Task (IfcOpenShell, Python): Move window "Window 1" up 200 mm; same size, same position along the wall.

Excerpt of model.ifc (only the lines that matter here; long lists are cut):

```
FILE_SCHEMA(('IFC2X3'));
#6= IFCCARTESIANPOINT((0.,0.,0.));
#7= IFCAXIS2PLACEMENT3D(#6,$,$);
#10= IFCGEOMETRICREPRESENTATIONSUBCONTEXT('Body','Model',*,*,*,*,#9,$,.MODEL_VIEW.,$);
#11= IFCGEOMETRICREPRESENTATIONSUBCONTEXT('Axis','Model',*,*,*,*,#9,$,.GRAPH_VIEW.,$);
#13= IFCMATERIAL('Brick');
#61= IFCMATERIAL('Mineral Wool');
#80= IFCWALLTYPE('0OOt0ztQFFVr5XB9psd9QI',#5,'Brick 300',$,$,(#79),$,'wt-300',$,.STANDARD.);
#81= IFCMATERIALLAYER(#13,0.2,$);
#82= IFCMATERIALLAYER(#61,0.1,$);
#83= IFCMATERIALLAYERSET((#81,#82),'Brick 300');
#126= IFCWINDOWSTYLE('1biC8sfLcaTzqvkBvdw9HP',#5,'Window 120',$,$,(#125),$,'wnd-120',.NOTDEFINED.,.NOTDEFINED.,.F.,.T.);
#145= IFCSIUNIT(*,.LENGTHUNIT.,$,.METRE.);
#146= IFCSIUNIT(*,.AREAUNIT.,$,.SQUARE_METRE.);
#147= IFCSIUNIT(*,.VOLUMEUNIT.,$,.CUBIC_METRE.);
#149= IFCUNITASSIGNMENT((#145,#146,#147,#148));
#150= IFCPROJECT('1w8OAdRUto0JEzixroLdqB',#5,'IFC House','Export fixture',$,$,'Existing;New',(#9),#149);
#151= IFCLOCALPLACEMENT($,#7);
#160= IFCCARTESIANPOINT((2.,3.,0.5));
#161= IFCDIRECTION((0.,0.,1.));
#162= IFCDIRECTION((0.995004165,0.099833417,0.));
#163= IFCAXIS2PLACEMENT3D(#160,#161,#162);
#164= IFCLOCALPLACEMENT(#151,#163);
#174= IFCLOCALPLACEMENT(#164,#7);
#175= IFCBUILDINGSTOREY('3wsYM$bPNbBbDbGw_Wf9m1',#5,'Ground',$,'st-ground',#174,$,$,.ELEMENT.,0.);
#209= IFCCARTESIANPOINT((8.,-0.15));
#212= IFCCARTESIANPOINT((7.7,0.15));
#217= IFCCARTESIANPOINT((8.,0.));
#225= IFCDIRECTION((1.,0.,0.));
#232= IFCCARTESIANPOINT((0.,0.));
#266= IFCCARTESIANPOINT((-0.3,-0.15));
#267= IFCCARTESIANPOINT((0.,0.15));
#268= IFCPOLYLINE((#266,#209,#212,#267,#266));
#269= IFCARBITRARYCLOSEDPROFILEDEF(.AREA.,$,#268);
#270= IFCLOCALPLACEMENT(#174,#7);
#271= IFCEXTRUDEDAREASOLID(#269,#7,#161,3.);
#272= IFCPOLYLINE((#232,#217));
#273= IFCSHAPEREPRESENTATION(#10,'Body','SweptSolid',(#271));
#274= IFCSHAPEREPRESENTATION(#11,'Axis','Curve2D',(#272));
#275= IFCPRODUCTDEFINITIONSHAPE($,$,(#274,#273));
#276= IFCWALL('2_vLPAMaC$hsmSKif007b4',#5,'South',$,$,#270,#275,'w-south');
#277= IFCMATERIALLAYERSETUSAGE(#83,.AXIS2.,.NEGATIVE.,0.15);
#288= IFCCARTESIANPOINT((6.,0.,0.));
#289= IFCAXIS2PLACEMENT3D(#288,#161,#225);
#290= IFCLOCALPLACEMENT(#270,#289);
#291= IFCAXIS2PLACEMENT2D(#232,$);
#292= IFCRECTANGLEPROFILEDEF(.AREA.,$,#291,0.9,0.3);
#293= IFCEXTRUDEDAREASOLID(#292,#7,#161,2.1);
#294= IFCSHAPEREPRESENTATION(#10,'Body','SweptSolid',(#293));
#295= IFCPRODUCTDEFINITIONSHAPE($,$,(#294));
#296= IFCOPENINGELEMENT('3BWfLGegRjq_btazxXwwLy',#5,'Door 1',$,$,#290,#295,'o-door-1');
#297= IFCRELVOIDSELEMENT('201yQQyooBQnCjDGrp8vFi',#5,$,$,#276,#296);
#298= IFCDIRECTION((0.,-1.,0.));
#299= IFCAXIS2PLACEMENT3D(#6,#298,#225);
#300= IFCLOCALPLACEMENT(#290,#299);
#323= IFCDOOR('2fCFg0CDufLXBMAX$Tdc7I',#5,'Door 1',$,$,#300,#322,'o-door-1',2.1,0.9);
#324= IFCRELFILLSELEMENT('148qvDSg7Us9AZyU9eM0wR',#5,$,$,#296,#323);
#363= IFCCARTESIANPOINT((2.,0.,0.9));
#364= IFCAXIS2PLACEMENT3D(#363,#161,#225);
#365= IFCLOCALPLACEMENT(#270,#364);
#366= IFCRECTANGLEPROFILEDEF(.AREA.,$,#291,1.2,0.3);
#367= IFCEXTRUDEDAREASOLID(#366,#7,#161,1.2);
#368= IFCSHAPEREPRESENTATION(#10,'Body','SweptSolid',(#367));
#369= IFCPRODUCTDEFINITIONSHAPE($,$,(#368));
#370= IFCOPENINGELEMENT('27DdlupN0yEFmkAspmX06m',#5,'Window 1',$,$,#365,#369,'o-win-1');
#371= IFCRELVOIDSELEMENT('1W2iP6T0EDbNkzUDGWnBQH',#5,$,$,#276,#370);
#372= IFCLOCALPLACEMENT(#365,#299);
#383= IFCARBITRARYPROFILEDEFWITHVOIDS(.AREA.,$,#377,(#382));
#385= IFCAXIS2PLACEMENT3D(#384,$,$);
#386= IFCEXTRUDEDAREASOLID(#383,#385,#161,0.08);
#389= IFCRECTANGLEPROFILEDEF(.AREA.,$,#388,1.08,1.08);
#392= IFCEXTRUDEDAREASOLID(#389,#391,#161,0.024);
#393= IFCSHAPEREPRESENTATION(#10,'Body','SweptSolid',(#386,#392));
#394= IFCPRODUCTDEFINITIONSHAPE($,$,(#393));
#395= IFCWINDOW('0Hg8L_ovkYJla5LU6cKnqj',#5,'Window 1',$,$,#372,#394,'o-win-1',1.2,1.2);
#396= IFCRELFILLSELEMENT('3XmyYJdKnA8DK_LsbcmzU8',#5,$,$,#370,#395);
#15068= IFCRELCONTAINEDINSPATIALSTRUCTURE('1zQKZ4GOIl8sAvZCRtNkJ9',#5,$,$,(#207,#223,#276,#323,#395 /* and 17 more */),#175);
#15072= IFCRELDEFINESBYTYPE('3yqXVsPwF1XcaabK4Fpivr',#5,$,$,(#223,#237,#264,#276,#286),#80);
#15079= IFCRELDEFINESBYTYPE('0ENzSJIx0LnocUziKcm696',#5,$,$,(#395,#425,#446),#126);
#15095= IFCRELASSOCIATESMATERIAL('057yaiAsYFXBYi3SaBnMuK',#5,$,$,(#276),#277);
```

```python
import numpy as np
import ifcopenshell
import ifcopenshell.api.geometry
import ifcopenshell.util.placement
import ifcopenshell.util.unit

model = ifcopenshell.open("model.ifc")
unit_scale = ifcopenshell.util.unit.calculate_unit_scale(model)

window = model.by_guid("0Hg8L_ovkYJla5LU6cKnqj")
opening = window.FillsVoids[0].RelatingOpeningElement
dz = 0.2 / unit_scale

shift = np.array([0.0, 0.0, dz])
# The window is placed relative to its opening, so it follows when the opening moves.
matrix = ifcopenshell.util.placement.get_local_placement(opening.ObjectPlacement)
matrix[:3, 3] += shift
ifcopenshell.api.geometry.edit_object_placement(
    model, product=opening, matrix=matrix, is_si=False, should_transform_children=True
)

print(f"moved by {dz * unit_scale:+.3f} m")

model.write("model-out.ifc")
```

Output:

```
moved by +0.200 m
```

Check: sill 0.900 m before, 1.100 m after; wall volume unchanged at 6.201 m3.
